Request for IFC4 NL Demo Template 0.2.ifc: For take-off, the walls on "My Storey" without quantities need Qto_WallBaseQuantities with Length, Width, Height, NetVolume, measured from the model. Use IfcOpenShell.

First a look at what the model holds.

```python
import ifcopenshell
import ifcopenshell.util.element
import ifcopenshell.util.unit

model = ifcopenshell.open("IFC4 NL Demo Template 0.2.ifc")
print(model.schema)
for unit_type in ("LENGTHUNIT", "AREAUNIT", "VOLUMEUNIT"):
    print(unit_type, ifcopenshell.util.unit.calculate_unit_scale(model, unit_type))
storey = next(s for s in model.by_type("IfcBuildingStorey") if s.Name == "My Storey")
walls = [e for e in ifcopenshell.util.element.get_decomposition(storey) if e.is_a("IfcWall")]
for e in sorted(walls, key=lambda e: e.id()):
    print(e.id(), e.is_a(), e.Name, list(ifcopenshell.util.element.get_psets(e, qtos_only=True)), sep=" | ")
```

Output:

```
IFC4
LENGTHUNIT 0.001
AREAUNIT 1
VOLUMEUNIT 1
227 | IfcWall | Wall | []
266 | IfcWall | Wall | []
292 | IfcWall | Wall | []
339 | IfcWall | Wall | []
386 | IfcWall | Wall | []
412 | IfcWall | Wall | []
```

```python
import ifcopenshell
import ifcopenshell.api.pset
import ifcopenshell.geom
import ifcopenshell.util.element
import ifcopenshell.util.shape
import ifcopenshell.util.unit

model = ifcopenshell.open("IFC4 NL Demo Template 0.2.ifc")
unit_scale = ifcopenshell.util.unit.calculate_unit_scale(model)
volume_scale = ifcopenshell.util.unit.calculate_unit_scale(model, "VOLUMEUNIT")
settings = ifcopenshell.geom.settings()

storey = next(s for s in model.by_type("IfcBuildingStorey") if s.Name == "My Storey")
walls = [e for e in ifcopenshell.util.element.get_decomposition(storey) if e.is_a("IfcWall")]

for e in sorted(walls, key=lambda e: e.id()):
    if ifcopenshell.util.element.get_psets(e, qtos_only=True, should_inherit=False):
        continue
    # Geometry comes back in metres, in the element's own axes.
    shape = ifcopenshell.geom.create_shape(settings, e)
    values = {
        "Length": ifcopenshell.util.shape.get_x(shape.geometry) / unit_scale,
        "Width": ifcopenshell.util.shape.get_y(shape.geometry) / unit_scale,
        "Height": ifcopenshell.util.shape.get_z(shape.geometry) / unit_scale,
        "NetVolume": ifcopenshell.util.shape.get_volume(shape.geometry) / volume_scale,
    }
    qto = ifcopenshell.api.pset.add_qto(model, product=e, name="Qto_WallBaseQuantities")
    ifcopenshell.api.pset.edit_qto(model, qto=qto, properties=values)
    print(e.id(), {k: round(v, 3) for k, v in values.items()})

model.write("IFC4 NL Demo Template 0.2-out.ifc")
```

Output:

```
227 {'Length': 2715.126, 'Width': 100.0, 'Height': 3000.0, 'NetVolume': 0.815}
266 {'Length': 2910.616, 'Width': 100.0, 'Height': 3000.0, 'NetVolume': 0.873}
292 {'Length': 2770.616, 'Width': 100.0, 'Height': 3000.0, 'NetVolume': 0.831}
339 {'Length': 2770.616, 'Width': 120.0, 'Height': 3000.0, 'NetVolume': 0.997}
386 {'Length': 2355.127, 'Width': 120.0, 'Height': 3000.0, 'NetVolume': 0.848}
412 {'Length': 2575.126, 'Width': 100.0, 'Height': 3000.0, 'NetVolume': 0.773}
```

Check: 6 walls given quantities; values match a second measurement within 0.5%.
